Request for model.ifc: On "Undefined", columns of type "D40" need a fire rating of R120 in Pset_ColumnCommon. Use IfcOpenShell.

First a look at what the model holds.

```python
import ifcopenshell
import ifcopenshell.util.element

model = ifcopenshell.open("model.ifc")
print(model.schema)
storey = next(s for s in model.by_type("IfcBuildingStorey") if s.Name == "Undefined")
columns = [e for e in ifcopenshell.util.element.get_decomposition(storey) if e.is_a("IfcColumn")]
seen = {}
for e in columns:
    element_type = ifcopenshell.util.element.get_type(e)
    key = (element_type.Name if element_type != e and element_type else None, ifcopenshell.util.element.get_pset(e, "Pset_ColumnCommon", "FireRating"))
    seen[key] = seen.get(key, 0) + 1
for (name, value), count in sorted(seen.items(), key=str):
    print(count, "x", name, "|", value)
```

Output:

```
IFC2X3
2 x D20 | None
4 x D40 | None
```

```python
import ifcopenshell
import ifcopenshell.api.pset
import ifcopenshell.util.element

model = ifcopenshell.open("model.ifc")

storey = next(s for s in model.by_type("IfcBuildingStorey") if s.Name == "Undefined")
columns = [e for e in ifcopenshell.util.element.get_decomposition(storey) if e.is_a("IfcColumn")]

count = 0
for e in columns:
    element_type = ifcopenshell.util.element.get_type(e)
    if element_type in (None, e) or element_type.Name != "D40":
        continue
    found = ifcopenshell.util.element.get_pset(e, "Pset_ColumnCommon", should_inherit=False)
    if found:
        pset = model.by_id(found["id"])
        if len(ifcopenshell.util.element.get_elements_by_pset(pset)) > 1:
            pset = ifcopenshell.api.pset.unshare_pset(model, products=[e], pset=pset)[0]
    else:
        pset = ifcopenshell.api.pset.add_pset(model, product=e, name="Pset_ColumnCommon")
    ifcopenshell.api.pset.edit_pset(model, pset=pset, properties={"FireRating": "R120"})
    count += 1

print(count, "columns updated")

model.write("model_v2.ifc")
```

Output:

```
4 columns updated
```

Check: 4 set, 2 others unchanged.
